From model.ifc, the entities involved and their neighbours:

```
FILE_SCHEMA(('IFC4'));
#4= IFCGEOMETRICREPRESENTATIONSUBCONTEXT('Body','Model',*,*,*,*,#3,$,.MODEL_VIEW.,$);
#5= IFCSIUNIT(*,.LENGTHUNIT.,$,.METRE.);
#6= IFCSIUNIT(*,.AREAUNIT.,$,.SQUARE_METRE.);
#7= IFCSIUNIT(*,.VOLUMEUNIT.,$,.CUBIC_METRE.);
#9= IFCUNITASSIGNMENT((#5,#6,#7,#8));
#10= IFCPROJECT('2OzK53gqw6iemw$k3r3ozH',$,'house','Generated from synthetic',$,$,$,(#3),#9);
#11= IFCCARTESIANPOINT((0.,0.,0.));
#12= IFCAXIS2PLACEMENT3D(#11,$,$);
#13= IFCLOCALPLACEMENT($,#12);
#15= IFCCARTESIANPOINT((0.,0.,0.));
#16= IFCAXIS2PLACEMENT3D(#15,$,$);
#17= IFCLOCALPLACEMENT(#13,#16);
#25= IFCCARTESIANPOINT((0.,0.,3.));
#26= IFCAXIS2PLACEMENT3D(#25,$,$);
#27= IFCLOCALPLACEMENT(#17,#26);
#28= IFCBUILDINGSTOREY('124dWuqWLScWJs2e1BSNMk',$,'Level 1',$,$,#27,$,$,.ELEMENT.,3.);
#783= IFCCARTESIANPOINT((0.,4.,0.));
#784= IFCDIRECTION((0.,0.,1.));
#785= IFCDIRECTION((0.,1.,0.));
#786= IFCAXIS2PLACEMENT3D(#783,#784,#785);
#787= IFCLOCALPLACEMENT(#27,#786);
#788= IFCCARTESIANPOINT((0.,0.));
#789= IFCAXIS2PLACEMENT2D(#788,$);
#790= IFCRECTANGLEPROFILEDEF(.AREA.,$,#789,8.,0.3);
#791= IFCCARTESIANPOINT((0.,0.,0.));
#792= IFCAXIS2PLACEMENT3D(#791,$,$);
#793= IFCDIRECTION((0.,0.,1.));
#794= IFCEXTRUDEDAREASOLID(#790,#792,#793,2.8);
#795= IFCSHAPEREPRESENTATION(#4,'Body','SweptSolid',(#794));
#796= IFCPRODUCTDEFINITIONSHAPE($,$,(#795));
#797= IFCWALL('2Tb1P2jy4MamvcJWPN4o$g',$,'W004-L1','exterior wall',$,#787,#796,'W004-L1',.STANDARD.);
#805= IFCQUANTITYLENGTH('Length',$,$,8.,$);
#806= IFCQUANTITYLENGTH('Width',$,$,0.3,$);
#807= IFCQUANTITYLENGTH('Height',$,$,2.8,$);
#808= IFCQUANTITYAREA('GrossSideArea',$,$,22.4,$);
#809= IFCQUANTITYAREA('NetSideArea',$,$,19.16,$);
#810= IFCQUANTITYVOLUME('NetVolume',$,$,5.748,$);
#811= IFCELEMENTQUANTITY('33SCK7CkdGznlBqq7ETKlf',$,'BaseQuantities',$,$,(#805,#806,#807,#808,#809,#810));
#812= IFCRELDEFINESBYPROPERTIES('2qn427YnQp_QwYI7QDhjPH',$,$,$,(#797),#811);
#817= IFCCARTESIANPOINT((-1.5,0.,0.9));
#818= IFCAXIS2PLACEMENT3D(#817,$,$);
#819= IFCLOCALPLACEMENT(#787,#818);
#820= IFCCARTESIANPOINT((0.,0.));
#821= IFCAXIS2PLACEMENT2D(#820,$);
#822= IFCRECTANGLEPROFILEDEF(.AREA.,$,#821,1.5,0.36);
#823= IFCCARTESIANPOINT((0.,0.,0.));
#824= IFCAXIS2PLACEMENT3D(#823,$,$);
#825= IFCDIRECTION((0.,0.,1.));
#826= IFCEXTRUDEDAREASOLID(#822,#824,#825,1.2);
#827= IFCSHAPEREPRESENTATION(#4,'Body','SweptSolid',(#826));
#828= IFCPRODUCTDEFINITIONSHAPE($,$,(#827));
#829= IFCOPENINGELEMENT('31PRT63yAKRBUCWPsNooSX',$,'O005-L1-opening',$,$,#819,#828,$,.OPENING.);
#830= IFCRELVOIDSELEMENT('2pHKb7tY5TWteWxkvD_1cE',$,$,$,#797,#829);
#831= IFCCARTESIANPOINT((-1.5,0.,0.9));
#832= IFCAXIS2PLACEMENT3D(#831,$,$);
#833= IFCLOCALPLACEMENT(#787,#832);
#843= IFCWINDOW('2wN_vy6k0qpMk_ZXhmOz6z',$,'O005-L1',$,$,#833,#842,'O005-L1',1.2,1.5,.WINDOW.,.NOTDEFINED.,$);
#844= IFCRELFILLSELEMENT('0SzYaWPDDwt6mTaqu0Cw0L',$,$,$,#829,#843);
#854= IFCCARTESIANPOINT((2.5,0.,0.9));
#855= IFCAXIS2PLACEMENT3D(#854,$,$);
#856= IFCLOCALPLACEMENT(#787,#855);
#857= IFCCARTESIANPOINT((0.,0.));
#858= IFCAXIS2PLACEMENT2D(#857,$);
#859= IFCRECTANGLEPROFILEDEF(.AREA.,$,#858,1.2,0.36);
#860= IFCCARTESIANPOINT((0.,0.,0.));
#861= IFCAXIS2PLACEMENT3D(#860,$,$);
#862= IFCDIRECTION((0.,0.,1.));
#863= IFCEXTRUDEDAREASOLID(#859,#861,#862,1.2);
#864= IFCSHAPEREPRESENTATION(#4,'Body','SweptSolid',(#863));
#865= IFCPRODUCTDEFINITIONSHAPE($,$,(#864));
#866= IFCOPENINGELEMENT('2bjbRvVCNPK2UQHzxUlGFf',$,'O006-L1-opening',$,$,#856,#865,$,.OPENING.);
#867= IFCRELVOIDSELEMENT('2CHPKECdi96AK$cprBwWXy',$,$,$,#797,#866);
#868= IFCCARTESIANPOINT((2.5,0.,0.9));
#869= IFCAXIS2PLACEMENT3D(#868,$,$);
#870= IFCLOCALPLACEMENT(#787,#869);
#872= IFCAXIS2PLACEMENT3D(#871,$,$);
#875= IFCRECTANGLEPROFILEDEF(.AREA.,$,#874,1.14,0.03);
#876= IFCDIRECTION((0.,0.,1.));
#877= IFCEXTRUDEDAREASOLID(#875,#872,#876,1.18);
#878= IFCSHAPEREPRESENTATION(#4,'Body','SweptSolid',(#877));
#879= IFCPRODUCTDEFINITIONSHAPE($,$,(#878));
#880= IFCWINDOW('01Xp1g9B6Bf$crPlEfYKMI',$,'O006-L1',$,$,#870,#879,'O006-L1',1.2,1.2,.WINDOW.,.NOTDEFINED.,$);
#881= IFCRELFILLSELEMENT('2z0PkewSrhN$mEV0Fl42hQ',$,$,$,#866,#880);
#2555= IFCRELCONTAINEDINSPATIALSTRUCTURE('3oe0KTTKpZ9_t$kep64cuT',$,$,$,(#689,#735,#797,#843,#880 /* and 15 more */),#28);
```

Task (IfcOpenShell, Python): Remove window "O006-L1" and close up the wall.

```python
import ifcopenshell
import ifcopenshell.api.feature
import ifcopenshell.api.pset
import ifcopenshell.api.root
import ifcopenshell.geom
import ifcopenshell.util.element
import ifcopenshell.util.shape
import ifcopenshell.util.unit

model = ifcopenshell.open("model.ifc")
area_scale = ifcopenshell.util.unit.calculate_unit_scale(model, "AREAUNIT")
volume_scale = ifcopenshell.util.unit.calculate_unit_scale(model, "VOLUMEUNIT")
settings = ifcopenshell.geom.settings()


def volume(element):
    """Net volume in cubic metres, openings subtracted."""
    shape = ifcopenshell.geom.create_shape(settings, element)
    return ifcopenshell.util.shape.get_volume(shape.geometry)


window = model.by_id(880)
opening = window.FillsVoids[0].RelatingOpeningElement
wall = opening.VoidsElements[0].RelatingBuildingElement
before = volume(wall)

ifcopenshell.api.root.remove_product(model, product=window)
ifcopenshell.api.feature.remove_feature(model, feature=opening)

after = volume(wall)
thickness = 0.3  # wall thickness in metres

# Update the wall's stored quantities.
qto = model.by_id(ifcopenshell.util.element.get_pset(wall, "BaseQuantities", should_inherit=False)["id"])
ifcopenshell.api.pset.edit_qto(model, qto=qto, properties={
    "NetSideArea": after / thickness / area_scale,
    "NetVolume": after / volume_scale,
})

print(f"wall volume {before:.3f} -> {after:.3f} m3")

model.write("model_edited.ifc")
```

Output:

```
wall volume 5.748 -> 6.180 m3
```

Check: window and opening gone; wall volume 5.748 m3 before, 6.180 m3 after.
